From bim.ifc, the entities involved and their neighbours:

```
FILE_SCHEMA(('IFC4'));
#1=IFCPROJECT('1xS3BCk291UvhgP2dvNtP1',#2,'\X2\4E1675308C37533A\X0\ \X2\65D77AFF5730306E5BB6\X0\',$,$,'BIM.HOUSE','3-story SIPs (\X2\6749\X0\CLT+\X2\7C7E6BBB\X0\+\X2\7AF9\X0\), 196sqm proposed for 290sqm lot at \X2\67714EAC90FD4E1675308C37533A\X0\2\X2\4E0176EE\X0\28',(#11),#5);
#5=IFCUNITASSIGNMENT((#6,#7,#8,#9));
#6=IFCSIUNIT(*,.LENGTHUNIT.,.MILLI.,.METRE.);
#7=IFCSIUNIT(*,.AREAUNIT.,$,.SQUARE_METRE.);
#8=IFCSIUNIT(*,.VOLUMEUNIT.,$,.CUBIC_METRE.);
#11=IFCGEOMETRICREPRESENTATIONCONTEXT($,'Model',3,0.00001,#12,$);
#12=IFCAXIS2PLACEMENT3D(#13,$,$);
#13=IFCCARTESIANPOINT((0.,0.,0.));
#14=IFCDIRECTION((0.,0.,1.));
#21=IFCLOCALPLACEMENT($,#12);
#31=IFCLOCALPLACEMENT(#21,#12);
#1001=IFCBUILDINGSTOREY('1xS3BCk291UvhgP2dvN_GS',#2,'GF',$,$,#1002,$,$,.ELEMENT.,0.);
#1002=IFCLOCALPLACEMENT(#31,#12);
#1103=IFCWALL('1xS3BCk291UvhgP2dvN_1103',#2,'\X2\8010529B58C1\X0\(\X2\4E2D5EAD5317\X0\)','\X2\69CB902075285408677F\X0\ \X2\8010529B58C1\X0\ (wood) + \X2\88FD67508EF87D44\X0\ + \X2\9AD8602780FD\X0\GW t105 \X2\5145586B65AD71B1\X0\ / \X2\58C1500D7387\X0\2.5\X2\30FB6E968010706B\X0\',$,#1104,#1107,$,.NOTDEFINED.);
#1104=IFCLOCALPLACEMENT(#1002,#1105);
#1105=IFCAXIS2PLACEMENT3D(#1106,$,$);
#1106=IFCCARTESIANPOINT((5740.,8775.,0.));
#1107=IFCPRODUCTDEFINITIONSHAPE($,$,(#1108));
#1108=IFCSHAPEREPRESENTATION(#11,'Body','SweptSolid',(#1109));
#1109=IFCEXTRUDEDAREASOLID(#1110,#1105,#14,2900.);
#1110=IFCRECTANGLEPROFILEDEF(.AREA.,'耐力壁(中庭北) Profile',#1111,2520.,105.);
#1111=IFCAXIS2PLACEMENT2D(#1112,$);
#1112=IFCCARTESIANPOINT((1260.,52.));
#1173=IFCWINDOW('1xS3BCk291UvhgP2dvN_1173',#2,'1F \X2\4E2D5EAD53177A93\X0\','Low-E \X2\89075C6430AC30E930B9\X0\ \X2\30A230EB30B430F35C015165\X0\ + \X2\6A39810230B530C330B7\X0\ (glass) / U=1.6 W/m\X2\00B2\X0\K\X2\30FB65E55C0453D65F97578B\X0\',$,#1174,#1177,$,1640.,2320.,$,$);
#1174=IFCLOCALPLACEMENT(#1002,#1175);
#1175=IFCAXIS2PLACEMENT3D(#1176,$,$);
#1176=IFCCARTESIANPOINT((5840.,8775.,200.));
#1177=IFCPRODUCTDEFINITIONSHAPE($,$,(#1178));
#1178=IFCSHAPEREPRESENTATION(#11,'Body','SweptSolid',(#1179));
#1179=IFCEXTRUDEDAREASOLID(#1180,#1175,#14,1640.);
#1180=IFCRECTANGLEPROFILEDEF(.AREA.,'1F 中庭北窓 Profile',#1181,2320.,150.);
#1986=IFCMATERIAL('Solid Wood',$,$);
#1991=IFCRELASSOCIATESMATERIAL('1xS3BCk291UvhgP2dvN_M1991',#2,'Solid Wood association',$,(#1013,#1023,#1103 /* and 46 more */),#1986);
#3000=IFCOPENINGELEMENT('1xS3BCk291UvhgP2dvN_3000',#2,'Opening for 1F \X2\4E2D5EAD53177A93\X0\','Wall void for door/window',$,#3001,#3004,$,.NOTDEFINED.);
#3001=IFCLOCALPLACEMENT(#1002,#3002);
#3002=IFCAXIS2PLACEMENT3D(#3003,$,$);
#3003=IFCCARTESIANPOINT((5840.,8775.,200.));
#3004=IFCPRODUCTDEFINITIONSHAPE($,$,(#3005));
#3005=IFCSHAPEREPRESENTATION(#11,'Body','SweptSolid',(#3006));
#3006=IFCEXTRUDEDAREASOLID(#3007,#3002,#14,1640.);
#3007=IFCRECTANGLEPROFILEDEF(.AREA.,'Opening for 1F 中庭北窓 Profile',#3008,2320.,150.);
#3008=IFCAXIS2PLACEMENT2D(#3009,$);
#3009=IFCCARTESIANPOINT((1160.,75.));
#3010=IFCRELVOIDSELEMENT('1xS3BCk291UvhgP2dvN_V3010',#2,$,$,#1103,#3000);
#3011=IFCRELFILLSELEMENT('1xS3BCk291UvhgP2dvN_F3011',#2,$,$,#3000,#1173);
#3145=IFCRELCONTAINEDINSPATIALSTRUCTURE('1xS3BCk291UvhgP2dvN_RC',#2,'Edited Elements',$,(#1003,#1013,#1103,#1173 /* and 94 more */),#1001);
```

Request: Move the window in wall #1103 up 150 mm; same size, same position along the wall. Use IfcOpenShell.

```python
import numpy as np
import ifcopenshell
import ifcopenshell.api.geometry
import ifcopenshell.util.placement
import ifcopenshell.util.unit

model = ifcopenshell.open("bim.ifc")
unit_scale = ifcopenshell.util.unit.calculate_unit_scale(model)

window = model.by_guid("1xS3BCk291UvhgP2dvN_1173")
opening = window.FillsVoids[0].RelatingOpeningElement
dz = 0.15 / unit_scale

shift = np.array([0.0, 0.0, dz])
# The window is not placed relative to its opening, so move both.
for product in (opening, window):
    matrix = ifcopenshell.util.placement.get_local_placement(product.ObjectPlacement)
    matrix[:3, 3] += shift
    ifcopenshell.api.geometry.edit_object_placement(model, product=product, matrix=matrix, is_si=False)

print(f"moved by {dz * unit_scale:+.3f} m")

model.write("bim-out.ifc")
```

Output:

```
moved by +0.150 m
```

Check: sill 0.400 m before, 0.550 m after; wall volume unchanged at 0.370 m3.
